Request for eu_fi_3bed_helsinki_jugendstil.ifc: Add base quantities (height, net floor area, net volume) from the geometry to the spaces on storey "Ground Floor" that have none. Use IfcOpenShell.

First a look at what the model holds.

```python
import ifcopenshell
import ifcopenshell.util.element
import ifcopenshell.util.unit

model = ifcopenshell.open("eu_fi_3bed_helsinki_jugendstil.ifc")
print(model.schema)
for unit_type in ("LENGTHUNIT", "AREAUNIT", "VOLUMEUNIT"):
    print(unit_type, ifcopenshell.util.unit.calculate_unit_scale(model, unit_type))
storey = next(s for s in model.by_type("IfcBuildingStorey") if s.Name == "Ground Floor")
spaces = [e for e in ifcopenshell.util.element.get_decomposition(storey) if e.is_a("IfcSpace")]
for e in sorted(spaces, key=lambda e: e.id()):
    print(e.id(), e.is_a(), e.Name, list(ifcopenshell.util.element.get_psets(e, qtos_only=True)), sep=" | ")
```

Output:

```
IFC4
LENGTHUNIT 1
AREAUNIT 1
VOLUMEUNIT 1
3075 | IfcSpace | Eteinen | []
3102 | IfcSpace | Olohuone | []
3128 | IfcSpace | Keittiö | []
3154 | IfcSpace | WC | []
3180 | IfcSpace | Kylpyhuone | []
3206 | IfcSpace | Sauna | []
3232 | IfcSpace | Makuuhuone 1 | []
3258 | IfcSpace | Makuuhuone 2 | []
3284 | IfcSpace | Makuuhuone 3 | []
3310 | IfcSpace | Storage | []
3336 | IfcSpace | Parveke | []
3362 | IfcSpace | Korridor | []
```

```python
import ifcopenshell
import ifcopenshell.api.pset
import ifcopenshell.geom
import ifcopenshell.util.element
import ifcopenshell.util.shape
import ifcopenshell.util.unit

model = ifcopenshell.open("eu_fi_3bed_helsinki_jugendstil.ifc")
unit_scale = ifcopenshell.util.unit.calculate_unit_scale(model)
area_scale = ifcopenshell.util.unit.calculate_unit_scale(model, "AREAUNIT")
volume_scale = ifcopenshell.util.unit.calculate_unit_scale(model, "VOLUMEUNIT")
settings = ifcopenshell.geom.settings()

storey = next(s for s in model.by_type("IfcBuildingStorey") if s.Name == "Ground Floor")
spaces = [e for e in ifcopenshell.util.element.get_decomposition(storey) if e.is_a("IfcSpace")]

for e in sorted(spaces, key=lambda e: e.id()):
    if ifcopenshell.util.element.get_psets(e, qtos_only=True, should_inherit=False):
        continue
    # Geometry comes back in metres, in the element's own axes.
    shape = ifcopenshell.geom.create_shape(settings, e)
    values = {
        "Height": ifcopenshell.util.shape.get_z(shape.geometry) / unit_scale,
        "NetFloorArea": ifcopenshell.util.shape.get_footprint_area(shape.geometry) / area_scale,
        "NetVolume": ifcopenshell.util.shape.get_volume(shape.geometry) / volume_scale,
    }
    qto = ifcopenshell.api.pset.add_qto(model, product=e, name="Qto_SpaceBaseQuantities")
    ifcopenshell.api.pset.edit_qto(model, qto=qto, properties=values)
    print(e.id(), {k: round(v, 3) for k, v in values.items()})

model.write("eu_fi_3bed_helsinki_jugendstil_rev.ifc")
```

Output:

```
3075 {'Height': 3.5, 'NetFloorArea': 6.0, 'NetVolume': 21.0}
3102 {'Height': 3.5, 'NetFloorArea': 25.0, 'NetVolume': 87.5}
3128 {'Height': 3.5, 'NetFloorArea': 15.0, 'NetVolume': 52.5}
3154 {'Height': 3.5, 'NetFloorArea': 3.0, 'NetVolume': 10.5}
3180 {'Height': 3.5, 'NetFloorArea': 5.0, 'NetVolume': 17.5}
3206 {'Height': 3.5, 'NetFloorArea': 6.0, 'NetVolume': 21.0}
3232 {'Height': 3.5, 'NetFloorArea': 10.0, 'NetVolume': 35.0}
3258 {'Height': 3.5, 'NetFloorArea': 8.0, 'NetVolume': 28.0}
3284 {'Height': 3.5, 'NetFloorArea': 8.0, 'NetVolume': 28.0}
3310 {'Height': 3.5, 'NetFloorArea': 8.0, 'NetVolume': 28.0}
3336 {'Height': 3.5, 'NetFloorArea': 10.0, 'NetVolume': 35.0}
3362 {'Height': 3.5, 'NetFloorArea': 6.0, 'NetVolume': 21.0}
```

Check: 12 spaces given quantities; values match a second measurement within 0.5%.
